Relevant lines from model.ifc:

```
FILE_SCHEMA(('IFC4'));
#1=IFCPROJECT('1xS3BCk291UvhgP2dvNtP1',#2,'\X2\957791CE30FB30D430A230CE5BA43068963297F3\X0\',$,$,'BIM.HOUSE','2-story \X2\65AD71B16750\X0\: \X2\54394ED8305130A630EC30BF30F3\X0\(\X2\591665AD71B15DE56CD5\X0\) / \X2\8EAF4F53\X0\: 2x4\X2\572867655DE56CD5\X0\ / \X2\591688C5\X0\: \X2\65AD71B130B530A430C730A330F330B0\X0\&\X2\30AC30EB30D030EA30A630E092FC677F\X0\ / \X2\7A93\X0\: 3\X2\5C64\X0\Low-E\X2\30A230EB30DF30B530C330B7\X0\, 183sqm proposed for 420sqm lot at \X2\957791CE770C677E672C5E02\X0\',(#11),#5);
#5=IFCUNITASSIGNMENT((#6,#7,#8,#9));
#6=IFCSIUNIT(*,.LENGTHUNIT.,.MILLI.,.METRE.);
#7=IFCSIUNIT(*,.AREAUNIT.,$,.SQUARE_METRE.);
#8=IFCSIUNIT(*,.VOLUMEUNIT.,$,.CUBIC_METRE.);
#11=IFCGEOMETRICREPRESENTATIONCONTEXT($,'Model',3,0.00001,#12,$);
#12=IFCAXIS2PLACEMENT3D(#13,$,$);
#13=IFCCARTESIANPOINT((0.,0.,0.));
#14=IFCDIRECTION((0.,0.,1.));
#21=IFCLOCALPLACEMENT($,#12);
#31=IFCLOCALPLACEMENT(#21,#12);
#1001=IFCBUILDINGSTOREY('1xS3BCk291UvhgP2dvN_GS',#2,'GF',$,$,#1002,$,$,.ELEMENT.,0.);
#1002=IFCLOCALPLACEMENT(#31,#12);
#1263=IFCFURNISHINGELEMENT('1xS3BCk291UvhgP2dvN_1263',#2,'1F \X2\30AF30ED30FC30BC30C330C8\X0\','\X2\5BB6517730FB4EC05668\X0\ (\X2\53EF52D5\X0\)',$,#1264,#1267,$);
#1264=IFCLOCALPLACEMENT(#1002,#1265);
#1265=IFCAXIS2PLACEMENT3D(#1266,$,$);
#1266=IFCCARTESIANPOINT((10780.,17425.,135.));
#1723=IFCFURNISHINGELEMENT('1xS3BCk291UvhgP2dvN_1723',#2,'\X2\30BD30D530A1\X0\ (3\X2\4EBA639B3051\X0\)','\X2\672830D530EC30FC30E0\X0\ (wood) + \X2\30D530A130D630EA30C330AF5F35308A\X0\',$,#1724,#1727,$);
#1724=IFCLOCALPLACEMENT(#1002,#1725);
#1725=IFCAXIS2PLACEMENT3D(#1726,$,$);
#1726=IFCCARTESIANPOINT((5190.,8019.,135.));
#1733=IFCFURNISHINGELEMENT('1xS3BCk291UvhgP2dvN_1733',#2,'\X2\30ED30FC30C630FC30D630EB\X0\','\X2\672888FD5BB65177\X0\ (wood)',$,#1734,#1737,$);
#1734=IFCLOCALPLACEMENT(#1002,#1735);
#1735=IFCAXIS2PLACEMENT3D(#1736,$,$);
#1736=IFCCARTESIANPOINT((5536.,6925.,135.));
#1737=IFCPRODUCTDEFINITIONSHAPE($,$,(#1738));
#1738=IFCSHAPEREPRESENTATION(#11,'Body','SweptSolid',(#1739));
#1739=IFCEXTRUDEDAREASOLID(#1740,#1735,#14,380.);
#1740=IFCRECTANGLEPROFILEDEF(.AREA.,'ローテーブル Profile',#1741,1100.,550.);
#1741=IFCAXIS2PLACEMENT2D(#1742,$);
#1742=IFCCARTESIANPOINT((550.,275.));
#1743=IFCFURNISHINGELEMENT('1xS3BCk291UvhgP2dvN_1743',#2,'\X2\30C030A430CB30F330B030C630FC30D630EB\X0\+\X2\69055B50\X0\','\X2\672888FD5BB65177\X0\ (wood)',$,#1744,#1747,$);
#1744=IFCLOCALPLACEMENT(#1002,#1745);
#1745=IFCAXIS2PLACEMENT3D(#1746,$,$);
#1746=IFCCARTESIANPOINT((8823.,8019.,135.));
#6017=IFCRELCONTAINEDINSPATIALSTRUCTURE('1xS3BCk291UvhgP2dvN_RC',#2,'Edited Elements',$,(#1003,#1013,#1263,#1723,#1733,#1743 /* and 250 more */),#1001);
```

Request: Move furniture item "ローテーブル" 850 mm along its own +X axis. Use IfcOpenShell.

```python
import ifcopenshell
import ifcopenshell.api.geometry
import ifcopenshell.util.placement

model = ifcopenshell.open("model.ifc")

item = model.by_guid("1xS3BCk291UvhgP2dvN_1733")
matrix = ifcopenshell.util.placement.get_local_placement(item.ObjectPlacement)
matrix[:3, 3] += matrix[:3, 0] * 850.0
ifcopenshell.api.geometry.edit_object_placement(model, product=item, matrix=matrix, is_si=False)

print(ifcopenshell.util.placement.get_local_placement(item.ObjectPlacement).round(3) + 0.0)

model.write("model_rev.ifc")
```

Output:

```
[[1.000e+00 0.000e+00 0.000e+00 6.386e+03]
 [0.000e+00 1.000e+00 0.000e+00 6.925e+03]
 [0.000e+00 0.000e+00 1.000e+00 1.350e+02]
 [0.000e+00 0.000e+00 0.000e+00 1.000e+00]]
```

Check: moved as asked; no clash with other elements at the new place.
